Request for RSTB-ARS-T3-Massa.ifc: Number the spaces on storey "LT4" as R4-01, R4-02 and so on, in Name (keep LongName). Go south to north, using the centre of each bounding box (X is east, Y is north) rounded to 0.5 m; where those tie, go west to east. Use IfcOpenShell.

First a look at what the model holds.

```python
import ifcopenshell
import ifcopenshell.util.element
import ifcopenshell.util.placement

model = ifcopenshell.open("RSTB-ARS-T3-Massa.ifc")
print(model.schema)
storey = next(s for s in model.by_type("IfcBuildingStorey") if s.Name == "LT4")
spaces = [e for e in ifcopenshell.util.element.get_decomposition(storey) if e.is_a("IfcSpace")]
for e in sorted(spaces, key=lambda e: e.id()):
    origin = ifcopenshell.util.placement.get_local_placement(e.ObjectPlacement)[:3, 3]
    print(e.id(), e.Name, e.LongName, origin.round(2) + 0.0, sep=" | ")
```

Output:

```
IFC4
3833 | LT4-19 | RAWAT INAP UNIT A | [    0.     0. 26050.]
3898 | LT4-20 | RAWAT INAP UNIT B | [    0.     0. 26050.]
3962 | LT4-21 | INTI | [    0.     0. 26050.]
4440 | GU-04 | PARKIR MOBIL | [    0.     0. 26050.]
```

```python
import ifcopenshell
import ifcopenshell.geom
import ifcopenshell.util.element
import ifcopenshell.util.shape

model = ifcopenshell.open("RSTB-ARS-T3-Massa.ifc")
settings = ifcopenshell.geom.settings()
settings.set("use-world-coords", True)


def centre(element):
    shape = ifcopenshell.geom.create_shape(settings, element)
    return ifcopenshell.util.shape.get_bbox_centroid(shape.geometry)


storey = next(s for s in model.by_type("IfcBuildingStorey") if s.Name == "LT4")
spaces = [e for e in ifcopenshell.util.element.get_decomposition(storey) if e.is_a("IfcSpace")]

# Insertion points can sit at a corner or the storey origin, so sort by the geometry (in metres).
centres = {e: centre(e) for e in spaces}
spaces.sort(key=lambda e: (round(centres[e][1] / 0.5), centres[e][0]))

for i, e in enumerate(spaces, start=1):
    number = f"R4-{i:02d}"
    e.Name = number
    print(e.id(), number)

model.write("RSTB-ARS-T3-Massa_rev.ifc")
```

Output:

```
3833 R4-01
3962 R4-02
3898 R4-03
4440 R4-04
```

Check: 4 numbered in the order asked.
